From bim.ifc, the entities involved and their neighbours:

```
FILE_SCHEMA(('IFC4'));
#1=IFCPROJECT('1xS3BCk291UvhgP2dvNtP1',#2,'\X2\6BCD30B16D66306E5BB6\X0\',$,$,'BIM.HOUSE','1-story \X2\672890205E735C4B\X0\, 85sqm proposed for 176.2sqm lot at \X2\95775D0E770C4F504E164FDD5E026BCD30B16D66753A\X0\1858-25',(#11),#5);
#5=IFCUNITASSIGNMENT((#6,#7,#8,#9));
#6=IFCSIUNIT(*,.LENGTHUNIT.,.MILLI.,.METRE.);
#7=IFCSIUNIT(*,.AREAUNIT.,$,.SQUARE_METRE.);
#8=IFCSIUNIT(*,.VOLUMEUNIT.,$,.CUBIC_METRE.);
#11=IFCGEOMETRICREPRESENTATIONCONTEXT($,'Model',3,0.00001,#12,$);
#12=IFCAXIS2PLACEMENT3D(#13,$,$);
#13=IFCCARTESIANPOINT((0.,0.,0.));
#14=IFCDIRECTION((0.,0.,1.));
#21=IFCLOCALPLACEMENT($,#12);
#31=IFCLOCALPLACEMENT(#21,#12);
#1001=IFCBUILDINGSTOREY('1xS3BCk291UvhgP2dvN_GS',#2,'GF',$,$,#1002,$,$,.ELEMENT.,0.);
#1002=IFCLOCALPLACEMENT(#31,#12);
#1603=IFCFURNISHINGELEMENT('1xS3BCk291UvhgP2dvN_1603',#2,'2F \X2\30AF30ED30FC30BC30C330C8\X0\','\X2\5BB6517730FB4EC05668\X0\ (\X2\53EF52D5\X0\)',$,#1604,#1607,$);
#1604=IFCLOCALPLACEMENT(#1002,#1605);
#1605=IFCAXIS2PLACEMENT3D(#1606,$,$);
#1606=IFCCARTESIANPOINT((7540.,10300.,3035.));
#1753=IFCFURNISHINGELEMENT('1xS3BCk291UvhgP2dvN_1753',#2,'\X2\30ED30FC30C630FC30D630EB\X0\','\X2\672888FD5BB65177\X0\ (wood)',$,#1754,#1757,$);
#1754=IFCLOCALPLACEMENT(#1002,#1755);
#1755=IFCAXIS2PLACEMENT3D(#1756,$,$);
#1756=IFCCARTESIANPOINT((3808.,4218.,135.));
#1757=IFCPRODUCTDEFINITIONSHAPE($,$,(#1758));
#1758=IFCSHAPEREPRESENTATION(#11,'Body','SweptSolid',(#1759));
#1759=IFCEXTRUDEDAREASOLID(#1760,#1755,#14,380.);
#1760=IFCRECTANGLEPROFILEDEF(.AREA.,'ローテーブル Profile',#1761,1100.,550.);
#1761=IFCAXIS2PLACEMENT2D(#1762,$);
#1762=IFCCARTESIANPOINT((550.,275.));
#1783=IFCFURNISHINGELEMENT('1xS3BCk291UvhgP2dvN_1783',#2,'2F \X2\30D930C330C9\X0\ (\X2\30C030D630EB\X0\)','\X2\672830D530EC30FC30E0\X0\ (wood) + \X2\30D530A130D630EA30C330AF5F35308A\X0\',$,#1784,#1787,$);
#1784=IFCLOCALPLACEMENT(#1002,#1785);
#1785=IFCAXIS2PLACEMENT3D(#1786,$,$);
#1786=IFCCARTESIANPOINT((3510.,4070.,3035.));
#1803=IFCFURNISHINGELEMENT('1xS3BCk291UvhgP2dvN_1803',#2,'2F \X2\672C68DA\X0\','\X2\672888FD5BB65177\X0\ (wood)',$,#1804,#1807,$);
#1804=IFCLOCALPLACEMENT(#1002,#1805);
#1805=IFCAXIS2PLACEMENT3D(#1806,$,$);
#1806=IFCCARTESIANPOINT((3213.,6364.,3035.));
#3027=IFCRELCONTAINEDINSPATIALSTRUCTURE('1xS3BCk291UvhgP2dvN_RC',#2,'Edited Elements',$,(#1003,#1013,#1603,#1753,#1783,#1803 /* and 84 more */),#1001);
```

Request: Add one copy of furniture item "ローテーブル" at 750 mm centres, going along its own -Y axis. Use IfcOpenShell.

```python
import ifcopenshell
import ifcopenshell.api.geometry
import ifcopenshell.api.root
import ifcopenshell.util.element
import ifcopenshell.util.placement

model = ifcopenshell.open("bim.ifc")


def reuse_history(source, copy):
    """copy_class also copies each property set's owner history, people and application; keep the originals."""
    for rel in copy.IsDefinedBy:
        if rel.is_a("IfcRelDefinesByProperties") and (history := rel.RelatingPropertyDefinition.OwnerHistory):
            rel.RelatingPropertyDefinition.OwnerHistory = source.OwnerHistory
            ifcopenshell.util.element.remove_deep2(model, history)


source = model.by_guid("1xS3BCk291UvhgP2dvN_1753")
base = ifcopenshell.util.placement.get_local_placement(source.ObjectPlacement)
step = -base[:3, 1] * 750.0

for i in range(1, 2):
    copy = ifcopenshell.api.root.copy_class(model, product=source)
    copy.Representation = ifcopenshell.util.element.copy_deep(
        model, source.Representation, exclude=["IfcGeometricRepresentationContext", "IfcRepresentationMap"]
    )
    reuse_history(source, copy)
    matrix = base.copy()
    matrix[:3, 3] += i * step
    print("added at", matrix[:3, 3].round(3) + 0.0)
    ifcopenshell.api.geometry.edit_object_placement(model, product=copy, matrix=matrix, is_si=False)

model.write("bim_updated.ifc")
```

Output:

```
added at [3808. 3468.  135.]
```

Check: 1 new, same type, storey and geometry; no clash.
